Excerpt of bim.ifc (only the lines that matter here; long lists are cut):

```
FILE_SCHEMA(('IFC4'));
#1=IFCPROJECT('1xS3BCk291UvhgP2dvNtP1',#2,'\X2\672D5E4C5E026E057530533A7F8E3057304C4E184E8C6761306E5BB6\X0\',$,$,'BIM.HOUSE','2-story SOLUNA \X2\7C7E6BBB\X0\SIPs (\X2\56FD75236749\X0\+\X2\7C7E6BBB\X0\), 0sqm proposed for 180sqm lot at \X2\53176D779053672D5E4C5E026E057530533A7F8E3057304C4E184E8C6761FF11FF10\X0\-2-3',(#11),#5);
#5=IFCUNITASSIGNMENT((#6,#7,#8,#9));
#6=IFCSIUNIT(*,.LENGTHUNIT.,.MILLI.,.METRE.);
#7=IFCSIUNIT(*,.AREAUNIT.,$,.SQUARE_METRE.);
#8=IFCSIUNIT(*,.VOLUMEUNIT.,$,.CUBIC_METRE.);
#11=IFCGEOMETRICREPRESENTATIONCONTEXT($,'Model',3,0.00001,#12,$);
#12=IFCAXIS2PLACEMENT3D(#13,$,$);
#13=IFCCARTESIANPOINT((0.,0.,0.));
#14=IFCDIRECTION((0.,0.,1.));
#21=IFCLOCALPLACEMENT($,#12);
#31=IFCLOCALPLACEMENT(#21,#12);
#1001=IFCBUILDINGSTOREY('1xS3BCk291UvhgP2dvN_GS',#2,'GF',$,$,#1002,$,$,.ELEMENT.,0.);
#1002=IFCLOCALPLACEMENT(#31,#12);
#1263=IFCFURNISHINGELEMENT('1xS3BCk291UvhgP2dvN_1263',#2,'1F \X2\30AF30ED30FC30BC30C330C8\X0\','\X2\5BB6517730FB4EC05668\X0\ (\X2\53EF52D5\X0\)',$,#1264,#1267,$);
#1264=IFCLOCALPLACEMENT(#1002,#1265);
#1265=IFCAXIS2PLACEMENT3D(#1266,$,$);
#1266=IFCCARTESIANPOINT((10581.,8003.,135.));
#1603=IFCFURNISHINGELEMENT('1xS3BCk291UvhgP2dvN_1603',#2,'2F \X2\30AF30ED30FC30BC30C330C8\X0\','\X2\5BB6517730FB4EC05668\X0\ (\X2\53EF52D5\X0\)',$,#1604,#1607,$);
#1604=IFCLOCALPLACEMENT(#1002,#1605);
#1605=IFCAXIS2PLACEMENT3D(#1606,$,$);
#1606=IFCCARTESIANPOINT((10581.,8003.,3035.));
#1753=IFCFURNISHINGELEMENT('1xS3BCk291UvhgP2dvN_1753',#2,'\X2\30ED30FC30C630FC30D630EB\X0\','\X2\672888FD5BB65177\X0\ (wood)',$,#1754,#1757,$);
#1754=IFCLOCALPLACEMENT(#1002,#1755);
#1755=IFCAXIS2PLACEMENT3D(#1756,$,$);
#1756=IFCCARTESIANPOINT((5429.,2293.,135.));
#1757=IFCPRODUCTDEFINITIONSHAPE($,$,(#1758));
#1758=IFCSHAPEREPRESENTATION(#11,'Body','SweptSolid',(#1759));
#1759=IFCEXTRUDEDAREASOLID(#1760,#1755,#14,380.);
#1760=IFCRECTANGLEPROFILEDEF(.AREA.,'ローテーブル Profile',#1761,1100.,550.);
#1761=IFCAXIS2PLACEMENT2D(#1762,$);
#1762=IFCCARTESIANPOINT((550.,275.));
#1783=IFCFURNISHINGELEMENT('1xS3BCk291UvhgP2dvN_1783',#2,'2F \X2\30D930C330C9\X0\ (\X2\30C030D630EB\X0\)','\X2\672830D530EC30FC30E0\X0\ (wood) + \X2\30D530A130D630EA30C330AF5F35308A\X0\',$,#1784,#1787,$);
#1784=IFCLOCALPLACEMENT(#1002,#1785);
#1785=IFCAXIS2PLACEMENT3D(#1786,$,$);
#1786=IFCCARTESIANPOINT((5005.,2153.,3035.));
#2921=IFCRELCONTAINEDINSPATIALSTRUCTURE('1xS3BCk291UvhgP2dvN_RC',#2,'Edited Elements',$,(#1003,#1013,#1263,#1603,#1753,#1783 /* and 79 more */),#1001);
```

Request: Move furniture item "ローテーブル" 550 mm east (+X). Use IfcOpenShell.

```python
import ifcopenshell
import ifcopenshell.api.geometry
import ifcopenshell.util.placement
import ifcopenshell.util.unit

model = ifcopenshell.open("bim.ifc")
unit_scale = ifcopenshell.util.unit.calculate_unit_scale(model)

item = model.by_guid("1xS3BCk291UvhgP2dvN_1753")
matrix = ifcopenshell.util.placement.get_local_placement(item.ObjectPlacement)
matrix[0, 3] += 0.55 / unit_scale
ifcopenshell.api.geometry.edit_object_placement(model, product=item, matrix=matrix, is_si=False)

print(ifcopenshell.util.placement.get_local_placement(item.ObjectPlacement).round(3) + 0.0)

model.write("bim_updated.ifc")
```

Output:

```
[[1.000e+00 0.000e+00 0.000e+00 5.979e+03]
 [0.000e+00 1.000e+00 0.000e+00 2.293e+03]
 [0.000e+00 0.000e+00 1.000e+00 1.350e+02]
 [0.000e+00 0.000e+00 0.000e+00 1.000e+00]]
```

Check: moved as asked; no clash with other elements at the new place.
